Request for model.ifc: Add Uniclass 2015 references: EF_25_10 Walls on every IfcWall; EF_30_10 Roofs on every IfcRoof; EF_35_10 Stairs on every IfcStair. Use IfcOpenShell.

First a look at what the model holds.

```python
import ifcopenshell

model = ifcopenshell.open("model.ifc")
print(model.schema)
print("classifications:", [c.Name for c in model.by_type("IfcClassification")])
for ifc_class in ("IfcDoor", "IfcRoof", "IfcStair", "IfcWall", "IfcWindow"):
    print(ifc_class, len(model.by_type(ifc_class)))
```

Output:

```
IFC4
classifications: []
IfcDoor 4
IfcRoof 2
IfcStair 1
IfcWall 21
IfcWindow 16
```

```python
import ifcopenshell
import ifcopenshell.api.classification

model = ifcopenshell.open("model.ifc")

system = ifcopenshell.api.classification.add_classification(model, classification="Uniclass 2015")

codes = {
    "IfcWall": ("EF_25_10", "Walls"),
    "IfcRoof": ("EF_30_10", "Roofs"),
    "IfcStair": ("EF_35_10", "Stairs"),
}
for ifc_class, (code, name) in codes.items():
    products = model.by_type(ifc_class)
    ifcopenshell.api.classification.add_reference(
        model, products=products, classification=system, identification=code, name=name
    )
    print(code, len(products))

model.write("model_updated.ifc")
```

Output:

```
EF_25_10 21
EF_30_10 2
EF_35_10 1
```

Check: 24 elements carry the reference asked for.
